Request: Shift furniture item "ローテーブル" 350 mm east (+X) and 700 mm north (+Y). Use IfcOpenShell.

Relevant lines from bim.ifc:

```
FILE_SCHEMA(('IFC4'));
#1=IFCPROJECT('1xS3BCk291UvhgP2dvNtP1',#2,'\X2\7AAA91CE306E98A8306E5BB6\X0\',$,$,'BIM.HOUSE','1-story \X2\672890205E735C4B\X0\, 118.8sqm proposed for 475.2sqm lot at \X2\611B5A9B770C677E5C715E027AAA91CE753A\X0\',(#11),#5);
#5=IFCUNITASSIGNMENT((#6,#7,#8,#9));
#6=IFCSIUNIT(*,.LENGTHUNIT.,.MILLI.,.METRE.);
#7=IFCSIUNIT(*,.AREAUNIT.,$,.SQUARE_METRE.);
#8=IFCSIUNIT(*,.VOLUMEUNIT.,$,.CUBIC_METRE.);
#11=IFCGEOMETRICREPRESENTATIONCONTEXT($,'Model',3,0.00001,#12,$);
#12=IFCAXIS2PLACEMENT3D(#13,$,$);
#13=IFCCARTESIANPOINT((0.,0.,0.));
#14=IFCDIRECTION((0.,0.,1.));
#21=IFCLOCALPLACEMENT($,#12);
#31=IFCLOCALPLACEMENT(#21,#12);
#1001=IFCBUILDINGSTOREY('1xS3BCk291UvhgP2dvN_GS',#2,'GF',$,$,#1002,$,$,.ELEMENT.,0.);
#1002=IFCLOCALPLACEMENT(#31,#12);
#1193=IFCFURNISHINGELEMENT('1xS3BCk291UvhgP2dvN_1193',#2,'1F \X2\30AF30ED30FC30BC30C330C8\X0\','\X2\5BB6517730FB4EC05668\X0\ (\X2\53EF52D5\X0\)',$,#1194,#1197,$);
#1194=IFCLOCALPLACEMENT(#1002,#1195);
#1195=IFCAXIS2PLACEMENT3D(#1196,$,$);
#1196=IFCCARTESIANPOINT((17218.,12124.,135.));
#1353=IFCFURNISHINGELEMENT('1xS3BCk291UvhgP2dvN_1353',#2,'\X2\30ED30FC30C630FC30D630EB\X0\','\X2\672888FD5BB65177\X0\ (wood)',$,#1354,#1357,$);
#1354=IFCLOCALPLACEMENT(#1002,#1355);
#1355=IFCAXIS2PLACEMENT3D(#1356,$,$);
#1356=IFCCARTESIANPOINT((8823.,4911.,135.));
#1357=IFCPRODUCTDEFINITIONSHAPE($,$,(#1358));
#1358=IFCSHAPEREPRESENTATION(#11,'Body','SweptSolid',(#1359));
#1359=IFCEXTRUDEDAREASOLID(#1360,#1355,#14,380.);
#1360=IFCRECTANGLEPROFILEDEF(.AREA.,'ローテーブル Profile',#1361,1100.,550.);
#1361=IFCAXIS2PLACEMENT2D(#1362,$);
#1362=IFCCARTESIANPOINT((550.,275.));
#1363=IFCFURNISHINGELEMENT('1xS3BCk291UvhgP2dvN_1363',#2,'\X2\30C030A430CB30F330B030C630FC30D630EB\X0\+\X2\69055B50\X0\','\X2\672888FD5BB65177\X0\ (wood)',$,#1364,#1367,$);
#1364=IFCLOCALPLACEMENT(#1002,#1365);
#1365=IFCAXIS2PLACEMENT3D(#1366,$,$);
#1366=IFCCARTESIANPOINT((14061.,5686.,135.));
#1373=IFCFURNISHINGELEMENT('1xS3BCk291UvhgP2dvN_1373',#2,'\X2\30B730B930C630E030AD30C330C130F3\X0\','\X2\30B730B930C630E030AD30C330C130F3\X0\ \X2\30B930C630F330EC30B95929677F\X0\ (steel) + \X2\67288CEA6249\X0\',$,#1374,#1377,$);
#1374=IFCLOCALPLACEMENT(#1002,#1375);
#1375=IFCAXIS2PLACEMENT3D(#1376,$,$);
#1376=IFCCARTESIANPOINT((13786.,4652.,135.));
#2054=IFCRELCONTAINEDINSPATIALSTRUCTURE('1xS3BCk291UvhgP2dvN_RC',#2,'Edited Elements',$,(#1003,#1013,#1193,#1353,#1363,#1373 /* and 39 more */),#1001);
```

```python
import ifcopenshell
import ifcopenshell.api.geometry
import ifcopenshell.util.placement

model = ifcopenshell.open("bim.ifc")

item = model.by_guid("1xS3BCk291UvhgP2dvN_1353")
matrix = ifcopenshell.util.placement.get_local_placement(item.ObjectPlacement)
matrix[0, 3] += 350.0
matrix[1, 3] += 700.0
ifcopenshell.api.geometry.edit_object_placement(model, product=item, matrix=matrix, is_si=False)

print(ifcopenshell.util.placement.get_local_placement(item.ObjectPlacement).round(3) + 0.0)

model.write("bim-out.ifc")
```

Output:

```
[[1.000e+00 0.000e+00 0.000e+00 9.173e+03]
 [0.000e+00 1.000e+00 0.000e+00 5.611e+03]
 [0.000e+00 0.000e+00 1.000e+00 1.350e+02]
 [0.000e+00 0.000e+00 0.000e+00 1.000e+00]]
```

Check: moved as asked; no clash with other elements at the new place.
